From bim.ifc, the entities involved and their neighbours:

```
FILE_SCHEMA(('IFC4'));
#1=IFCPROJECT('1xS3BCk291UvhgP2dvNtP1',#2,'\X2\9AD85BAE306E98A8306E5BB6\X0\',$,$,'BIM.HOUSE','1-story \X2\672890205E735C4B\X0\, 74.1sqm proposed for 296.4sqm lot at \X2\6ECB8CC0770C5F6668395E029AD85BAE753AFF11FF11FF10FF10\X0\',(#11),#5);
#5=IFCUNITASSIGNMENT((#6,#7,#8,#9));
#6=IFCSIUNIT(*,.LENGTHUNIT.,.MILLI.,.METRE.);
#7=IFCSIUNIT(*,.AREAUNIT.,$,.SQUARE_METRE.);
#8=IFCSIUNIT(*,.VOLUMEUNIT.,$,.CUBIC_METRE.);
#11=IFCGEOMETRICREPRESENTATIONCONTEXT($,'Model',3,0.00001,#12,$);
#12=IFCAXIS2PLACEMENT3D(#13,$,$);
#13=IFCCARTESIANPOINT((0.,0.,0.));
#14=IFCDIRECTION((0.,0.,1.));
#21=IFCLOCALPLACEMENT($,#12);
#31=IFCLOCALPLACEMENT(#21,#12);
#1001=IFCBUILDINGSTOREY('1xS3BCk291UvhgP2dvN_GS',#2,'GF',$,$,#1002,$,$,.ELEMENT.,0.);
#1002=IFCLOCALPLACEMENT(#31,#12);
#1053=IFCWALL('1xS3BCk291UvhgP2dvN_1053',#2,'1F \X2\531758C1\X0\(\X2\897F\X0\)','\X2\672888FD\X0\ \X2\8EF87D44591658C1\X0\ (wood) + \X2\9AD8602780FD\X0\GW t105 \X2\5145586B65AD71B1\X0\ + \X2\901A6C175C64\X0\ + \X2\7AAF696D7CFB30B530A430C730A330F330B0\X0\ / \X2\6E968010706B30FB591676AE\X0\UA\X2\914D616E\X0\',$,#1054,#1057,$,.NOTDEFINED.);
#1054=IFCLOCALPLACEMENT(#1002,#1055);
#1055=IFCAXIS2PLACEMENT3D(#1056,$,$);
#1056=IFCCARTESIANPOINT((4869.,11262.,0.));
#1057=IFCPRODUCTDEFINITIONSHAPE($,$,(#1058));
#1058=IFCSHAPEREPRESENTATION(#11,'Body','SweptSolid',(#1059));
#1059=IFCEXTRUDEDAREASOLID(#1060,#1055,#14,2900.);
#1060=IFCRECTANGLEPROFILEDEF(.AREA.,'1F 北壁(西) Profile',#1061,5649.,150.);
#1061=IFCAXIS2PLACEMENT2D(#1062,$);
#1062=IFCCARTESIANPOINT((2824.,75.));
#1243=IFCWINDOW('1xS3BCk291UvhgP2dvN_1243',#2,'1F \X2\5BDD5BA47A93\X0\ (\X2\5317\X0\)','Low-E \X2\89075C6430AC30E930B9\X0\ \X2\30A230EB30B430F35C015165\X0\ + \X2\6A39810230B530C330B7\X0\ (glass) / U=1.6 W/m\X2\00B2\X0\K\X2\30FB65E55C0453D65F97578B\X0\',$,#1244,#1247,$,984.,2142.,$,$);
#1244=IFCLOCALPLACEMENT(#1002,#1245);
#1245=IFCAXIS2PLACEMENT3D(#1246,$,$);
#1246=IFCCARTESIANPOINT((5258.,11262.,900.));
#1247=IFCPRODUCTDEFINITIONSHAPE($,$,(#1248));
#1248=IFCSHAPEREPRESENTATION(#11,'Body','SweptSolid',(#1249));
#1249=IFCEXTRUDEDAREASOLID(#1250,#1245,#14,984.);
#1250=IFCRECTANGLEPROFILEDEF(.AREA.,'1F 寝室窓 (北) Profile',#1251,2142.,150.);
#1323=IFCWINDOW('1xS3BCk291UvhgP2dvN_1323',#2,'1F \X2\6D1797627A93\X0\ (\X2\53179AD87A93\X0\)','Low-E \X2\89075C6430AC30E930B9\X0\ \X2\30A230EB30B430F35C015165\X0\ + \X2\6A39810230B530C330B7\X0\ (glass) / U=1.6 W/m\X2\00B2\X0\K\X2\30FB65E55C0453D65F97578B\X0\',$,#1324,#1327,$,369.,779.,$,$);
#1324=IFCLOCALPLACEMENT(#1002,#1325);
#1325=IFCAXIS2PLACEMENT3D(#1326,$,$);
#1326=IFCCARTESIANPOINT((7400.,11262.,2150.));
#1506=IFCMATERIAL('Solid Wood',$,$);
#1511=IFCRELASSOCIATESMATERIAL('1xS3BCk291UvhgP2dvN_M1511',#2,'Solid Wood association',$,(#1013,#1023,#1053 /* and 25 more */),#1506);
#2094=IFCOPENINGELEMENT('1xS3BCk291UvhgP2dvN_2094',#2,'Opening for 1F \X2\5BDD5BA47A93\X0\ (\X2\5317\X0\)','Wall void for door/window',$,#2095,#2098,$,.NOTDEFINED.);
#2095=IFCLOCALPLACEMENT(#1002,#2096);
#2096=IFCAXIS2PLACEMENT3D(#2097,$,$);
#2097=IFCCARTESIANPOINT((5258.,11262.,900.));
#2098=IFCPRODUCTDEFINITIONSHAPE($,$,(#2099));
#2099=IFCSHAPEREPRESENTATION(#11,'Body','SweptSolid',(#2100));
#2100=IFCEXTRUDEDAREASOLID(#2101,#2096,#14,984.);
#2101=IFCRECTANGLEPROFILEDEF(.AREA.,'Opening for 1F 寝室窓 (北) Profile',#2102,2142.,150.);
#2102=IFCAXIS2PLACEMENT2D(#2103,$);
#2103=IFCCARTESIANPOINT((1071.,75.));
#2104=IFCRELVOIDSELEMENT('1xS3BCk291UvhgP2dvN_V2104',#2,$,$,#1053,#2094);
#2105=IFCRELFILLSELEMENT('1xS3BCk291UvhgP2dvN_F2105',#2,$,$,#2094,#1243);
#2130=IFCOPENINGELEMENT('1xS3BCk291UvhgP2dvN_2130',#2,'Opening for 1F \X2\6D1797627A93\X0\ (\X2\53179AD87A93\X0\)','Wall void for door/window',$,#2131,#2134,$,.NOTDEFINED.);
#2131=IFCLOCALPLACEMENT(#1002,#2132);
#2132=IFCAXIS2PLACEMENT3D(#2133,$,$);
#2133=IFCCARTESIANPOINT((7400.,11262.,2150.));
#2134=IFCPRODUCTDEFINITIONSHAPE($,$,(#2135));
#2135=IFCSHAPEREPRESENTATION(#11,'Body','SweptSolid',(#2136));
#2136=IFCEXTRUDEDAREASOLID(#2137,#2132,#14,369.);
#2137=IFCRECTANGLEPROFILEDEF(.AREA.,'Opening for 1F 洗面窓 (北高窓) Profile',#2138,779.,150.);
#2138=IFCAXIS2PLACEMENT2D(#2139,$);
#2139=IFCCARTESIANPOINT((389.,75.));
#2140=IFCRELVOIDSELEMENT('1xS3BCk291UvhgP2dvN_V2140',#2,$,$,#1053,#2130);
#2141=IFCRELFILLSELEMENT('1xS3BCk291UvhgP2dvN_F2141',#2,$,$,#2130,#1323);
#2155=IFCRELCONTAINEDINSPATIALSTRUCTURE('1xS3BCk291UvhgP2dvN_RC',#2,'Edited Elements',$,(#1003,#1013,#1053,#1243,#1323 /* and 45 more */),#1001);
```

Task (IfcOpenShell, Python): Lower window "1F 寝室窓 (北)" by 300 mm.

```python
import numpy as np
import ifcopenshell
import ifcopenshell.api.geometry
import ifcopenshell.util.placement
import ifcopenshell.util.unit

model = ifcopenshell.open("bim.ifc")
unit_scale = ifcopenshell.util.unit.calculate_unit_scale(model)

window = model.by_id(1243)
opening = window.FillsVoids[0].RelatingOpeningElement
dz = -0.3 / unit_scale

shift = np.array([0.0, 0.0, dz])
# The window is not placed relative to its opening, so move both.
for product in (opening, window):
    matrix = ifcopenshell.util.placement.get_local_placement(product.ObjectPlacement)
    matrix[:3, 3] += shift
    ifcopenshell.api.geometry.edit_object_placement(model, product=product, matrix=matrix, is_si=False)

print(f"moved by {dz * unit_scale:+.3f} m")

model.write("bim_edited.ifc")
```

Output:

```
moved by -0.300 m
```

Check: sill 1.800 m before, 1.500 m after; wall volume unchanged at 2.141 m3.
